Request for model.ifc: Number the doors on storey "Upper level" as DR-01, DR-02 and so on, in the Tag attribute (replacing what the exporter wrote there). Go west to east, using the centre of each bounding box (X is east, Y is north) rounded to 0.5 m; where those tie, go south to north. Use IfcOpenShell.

First a look at what the model holds.

```python
import ifcopenshell
import ifcopenshell.util.element
import ifcopenshell.util.placement

model = ifcopenshell.open("model.ifc")
print(model.schema)
storey = next(s for s in model.by_type("IfcBuildingStorey") if s.Name == "Upper level")
doors = [e for e in ifcopenshell.util.element.get_decomposition(storey) if e.is_a("IfcDoor")]
for e in sorted(doors, key=lambda e: e.id()):
    origin = ifcopenshell.util.placement.get_local_placement(e.ObjectPlacement)[:3, 3]
    print(e.id(), e.Tag, e.Name, origin.round(2) + 0.0, sep=" | ")
```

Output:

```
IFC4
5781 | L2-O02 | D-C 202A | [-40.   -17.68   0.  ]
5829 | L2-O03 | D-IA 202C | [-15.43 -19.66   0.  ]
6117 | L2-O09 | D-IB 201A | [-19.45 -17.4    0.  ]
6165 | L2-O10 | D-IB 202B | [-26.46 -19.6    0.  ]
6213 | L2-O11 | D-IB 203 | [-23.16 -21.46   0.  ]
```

```python
import ifcopenshell
import ifcopenshell.geom
import ifcopenshell.util.element
import ifcopenshell.util.shape

model = ifcopenshell.open("model.ifc")
settings = ifcopenshell.geom.settings()
settings.set("use-world-coords", True)


def centre(element):
    shape = ifcopenshell.geom.create_shape(settings, element)
    return ifcopenshell.util.shape.get_bbox_centroid(shape.geometry)


storey = next(s for s in model.by_type("IfcBuildingStorey") if s.Name == "Upper level")
doors = [e for e in ifcopenshell.util.element.get_decomposition(storey) if e.is_a("IfcDoor")]

# Insertion points can sit at a corner or the storey origin, so sort by the geometry (in metres).
centres = {e: centre(e) for e in doors}
doors.sort(key=lambda e: (round(centres[e][0] / 0.5), centres[e][1]))

for i, e in enumerate(doors, start=1):
    number = f"DR-{i:02d}"
    e.Tag = number
    print(e.id(), number)

model.write("model_rev.ifc")
```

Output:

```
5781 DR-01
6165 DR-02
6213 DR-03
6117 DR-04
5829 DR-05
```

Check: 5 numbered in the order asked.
